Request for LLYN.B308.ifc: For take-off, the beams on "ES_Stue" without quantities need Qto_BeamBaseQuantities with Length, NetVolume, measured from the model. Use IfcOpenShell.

First a look at what the model holds.

```python
import ifcopenshell
import ifcopenshell.util.element
import ifcopenshell.util.unit

model = ifcopenshell.open("LLYN.B308.ifc")
print(model.schema)
for unit_type in ("LENGTHUNIT", "AREAUNIT", "VOLUMEUNIT"):
    print(unit_type, ifcopenshell.util.unit.calculate_unit_scale(model, unit_type))
storey = next(s for s in model.by_type("IfcBuildingStorey") if s.Name == "ES_Stue")
beams = [e for e in ifcopenshell.util.element.get_decomposition(storey) if e.is_a("IfcBeam")]
for e in sorted(beams, key=lambda e: e.id()):
    print(e.id(), e.is_a(), e.Name, list(ifcopenshell.util.element.get_psets(e, qtos_only=True)), sep=" | ")
```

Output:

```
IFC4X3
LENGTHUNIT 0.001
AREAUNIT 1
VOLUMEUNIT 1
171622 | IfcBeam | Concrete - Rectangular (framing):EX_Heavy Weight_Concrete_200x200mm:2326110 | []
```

```python
import ifcopenshell
import ifcopenshell.api.pset
import ifcopenshell.geom
import ifcopenshell.util.element
import ifcopenshell.util.shape
import ifcopenshell.util.unit

model = ifcopenshell.open("LLYN.B308.ifc")
unit_scale = ifcopenshell.util.unit.calculate_unit_scale(model)
volume_scale = ifcopenshell.util.unit.calculate_unit_scale(model, "VOLUMEUNIT")
settings = ifcopenshell.geom.settings()

storey = next(s for s in model.by_type("IfcBuildingStorey") if s.Name == "ES_Stue")
beams = [e for e in ifcopenshell.util.element.get_decomposition(storey) if e.is_a("IfcBeam")]

for e in sorted(beams, key=lambda e: e.id()):
    if ifcopenshell.util.element.get_psets(e, qtos_only=True, should_inherit=False):
        continue
    # Geometry comes back in metres, in the element's own axes.
    shape = ifcopenshell.geom.create_shape(settings, e)
    values = {
        "Length": ifcopenshell.util.shape.get_max_xyz(shape.geometry) / unit_scale,
        "NetVolume": ifcopenshell.util.shape.get_volume(shape.geometry) / volume_scale,
    }
    qto = ifcopenshell.api.pset.add_qto(model, product=e, name="Qto_BeamBaseQuantities")
    ifcopenshell.api.pset.edit_qto(model, qto=qto, properties=values)
    print(e.id(), {k: round(v, 3) for k, v in values.items()})

model.write("LLYN.B308_updated.ifc")
```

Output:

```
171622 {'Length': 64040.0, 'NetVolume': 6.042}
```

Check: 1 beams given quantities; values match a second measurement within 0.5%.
